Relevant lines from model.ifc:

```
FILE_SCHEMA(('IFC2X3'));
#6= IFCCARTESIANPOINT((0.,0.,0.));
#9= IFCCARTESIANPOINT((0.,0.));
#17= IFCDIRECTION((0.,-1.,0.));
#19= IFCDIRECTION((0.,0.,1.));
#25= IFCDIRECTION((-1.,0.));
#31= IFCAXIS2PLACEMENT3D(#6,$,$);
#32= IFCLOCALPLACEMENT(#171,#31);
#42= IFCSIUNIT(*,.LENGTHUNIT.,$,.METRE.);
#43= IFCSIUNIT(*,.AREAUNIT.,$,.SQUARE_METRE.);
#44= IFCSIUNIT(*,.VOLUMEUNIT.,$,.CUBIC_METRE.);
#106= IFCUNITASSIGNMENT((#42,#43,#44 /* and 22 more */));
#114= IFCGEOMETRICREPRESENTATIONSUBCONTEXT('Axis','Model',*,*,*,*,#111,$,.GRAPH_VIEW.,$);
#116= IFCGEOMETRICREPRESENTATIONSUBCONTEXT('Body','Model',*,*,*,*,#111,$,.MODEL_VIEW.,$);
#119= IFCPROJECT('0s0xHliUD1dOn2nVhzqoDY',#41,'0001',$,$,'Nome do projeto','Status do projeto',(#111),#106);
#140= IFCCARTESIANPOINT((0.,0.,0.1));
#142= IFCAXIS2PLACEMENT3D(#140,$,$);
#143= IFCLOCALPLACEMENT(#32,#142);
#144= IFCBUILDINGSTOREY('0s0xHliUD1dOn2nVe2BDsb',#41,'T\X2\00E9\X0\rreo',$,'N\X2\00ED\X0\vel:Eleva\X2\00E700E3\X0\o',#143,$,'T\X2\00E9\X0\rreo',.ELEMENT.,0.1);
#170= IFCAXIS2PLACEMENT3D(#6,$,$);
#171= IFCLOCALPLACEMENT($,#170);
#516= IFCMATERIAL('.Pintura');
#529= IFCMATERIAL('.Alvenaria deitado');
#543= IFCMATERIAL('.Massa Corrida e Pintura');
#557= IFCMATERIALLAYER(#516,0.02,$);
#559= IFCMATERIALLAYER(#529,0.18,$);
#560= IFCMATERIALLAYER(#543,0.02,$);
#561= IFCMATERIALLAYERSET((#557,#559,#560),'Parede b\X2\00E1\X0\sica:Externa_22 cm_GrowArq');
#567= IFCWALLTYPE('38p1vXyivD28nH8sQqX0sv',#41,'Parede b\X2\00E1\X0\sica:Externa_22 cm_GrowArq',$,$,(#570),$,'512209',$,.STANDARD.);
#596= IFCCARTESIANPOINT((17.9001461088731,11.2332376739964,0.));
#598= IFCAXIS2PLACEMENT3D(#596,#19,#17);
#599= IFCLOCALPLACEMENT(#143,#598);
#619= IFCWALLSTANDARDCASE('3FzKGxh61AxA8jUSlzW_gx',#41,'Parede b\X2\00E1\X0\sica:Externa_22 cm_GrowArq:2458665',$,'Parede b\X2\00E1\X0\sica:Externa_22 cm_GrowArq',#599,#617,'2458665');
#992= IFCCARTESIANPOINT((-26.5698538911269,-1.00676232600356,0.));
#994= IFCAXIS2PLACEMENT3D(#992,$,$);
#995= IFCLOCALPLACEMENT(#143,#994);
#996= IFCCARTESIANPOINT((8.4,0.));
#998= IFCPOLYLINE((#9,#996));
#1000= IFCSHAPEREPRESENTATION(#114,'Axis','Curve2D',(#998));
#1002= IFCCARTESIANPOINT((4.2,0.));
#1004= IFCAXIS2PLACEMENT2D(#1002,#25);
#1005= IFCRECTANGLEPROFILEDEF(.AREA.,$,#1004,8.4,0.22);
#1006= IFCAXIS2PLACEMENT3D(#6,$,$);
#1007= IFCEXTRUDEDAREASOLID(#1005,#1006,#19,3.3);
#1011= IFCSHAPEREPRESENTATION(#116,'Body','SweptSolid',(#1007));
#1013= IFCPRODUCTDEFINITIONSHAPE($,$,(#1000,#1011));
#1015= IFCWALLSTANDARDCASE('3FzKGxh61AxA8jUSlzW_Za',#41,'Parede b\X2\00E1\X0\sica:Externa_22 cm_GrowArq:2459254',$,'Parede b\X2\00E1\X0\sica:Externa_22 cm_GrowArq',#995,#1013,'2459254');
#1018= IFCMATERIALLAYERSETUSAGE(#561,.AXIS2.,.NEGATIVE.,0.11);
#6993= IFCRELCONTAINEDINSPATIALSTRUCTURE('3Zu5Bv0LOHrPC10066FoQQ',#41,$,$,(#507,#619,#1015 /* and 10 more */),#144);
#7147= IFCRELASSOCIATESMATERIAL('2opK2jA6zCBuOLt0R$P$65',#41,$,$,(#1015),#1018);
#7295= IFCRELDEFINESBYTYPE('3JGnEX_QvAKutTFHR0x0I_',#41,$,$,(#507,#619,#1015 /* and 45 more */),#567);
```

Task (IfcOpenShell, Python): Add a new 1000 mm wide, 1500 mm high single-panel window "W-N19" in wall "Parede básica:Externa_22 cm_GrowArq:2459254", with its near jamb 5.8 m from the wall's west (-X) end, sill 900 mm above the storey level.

```python
import numpy as np
import ifcopenshell
import ifcopenshell.api.feature
import ifcopenshell.api.geometry
import ifcopenshell.api.root
import ifcopenshell.api.spatial
import ifcopenshell.api.type
import ifcopenshell.geom
import ifcopenshell.util.element
import ifcopenshell.util.placement
import ifcopenshell.util.representation
import ifcopenshell.util.shape
import ifcopenshell.util.unit

model = ifcopenshell.open("model.ifc")
unit_scale = ifcopenshell.util.unit.calculate_unit_scale(model)
settings = ifcopenshell.geom.settings()


def volume(element):
    """Net volume in cubic metres, openings subtracted."""
    shape = ifcopenshell.geom.create_shape(settings, element)
    return ifcopenshell.util.shape.get_volume(shape.geometry)


wall = model.by_guid("3FzKGxh61AxA8jUSlzW_Za")
storey = ifcopenshell.util.element.get_container(wall, ifc_class="IfcBuildingStorey")
context = ifcopenshell.util.representation.get_context(model, "Model", "Body", "MODEL_VIEW")
before = volume(wall)

width, height, from_end, sill = 1, 1.5, 5.8, 0.9  # metres

# The wall runs along its own X axis, and the end named is its -X end.
wall_shape = ifcopenshell.geom.create_shape(settings, wall)
x, y, z = ifcopenshell.util.shape.get_vertices(wall_shape.geometry).T
start = x.min() + from_end
face, thickness = float(y.min()), float(y.max() - y.min())
wall_matrix = ifcopenshell.util.placement.get_local_placement(wall.ObjectPlacement)
level = ifcopenshell.util.placement.get_local_placement(storey.ObjectPlacement)[2, 3]


def in_wall(x, y):
    """Placement at x, y metres in the wall's axes, at sill height."""
    matrix = wall_matrix.copy()
    matrix[:, 3] = wall_matrix @ np.array([x / unit_scale, y / unit_scale, 0.0, 1.0])
    matrix[2, 3] = level + sill / unit_scale
    return matrix


# Opening: a box that overshoots both wall faces by 50 mm.
opening = ifcopenshell.api.root.create_entity(model, ifc_class="IfcOpeningElement")
box = ifcopenshell.api.geometry.add_wall_representation(
    model, context=context, length=width, height=height, thickness=thickness + 0.1
)
ifcopenshell.api.geometry.assign_representation(model, product=opening, representation=box)
ifcopenshell.api.geometry.edit_object_placement(model, product=opening, matrix=in_wall(start, face - 0.05), is_si=False)
ifcopenshell.api.feature.add_feature(model, feature=opening, element=wall)

window = ifcopenshell.api.root.create_entity(model, ifc_class="IfcWindow", name="W-N19")
window.OverallWidth, window.OverallHeight = width / unit_scale, height / unit_scale
body = ifcopenshell.api.geometry.add_window_representation(
    model,
    context=context,
    overall_width=window.OverallWidth,
    overall_height=window.OverallHeight,
    partition_type="SINGLE_PANEL",
)
ifcopenshell.api.geometry.assign_representation(model, product=window, representation=body)
ifcopenshell.api.spatial.assign_container(model, products=[window], relating_structure=storey)
fills = ifcopenshell.api.feature.add_filling(model, opening=opening, element=window)
fills.OwnerHistory = window.OwnerHistory  # required in IFC2X3

# IFC2X3 keeps the operation on the window style.
style = ifcopenshell.api.root.create_entity(model, ifc_class="IfcWindowStyle", name="W-N19")
style.OperationType, style.ConstructionType = "SINGLE_PANEL", "NOTDEFINED"
style.ParameterTakesPrecedence = style.Sizeable = False
ifcopenshell.api.type.assign_type(model, related_objects=[window], relating_type=style)

# Centre the window in the wall's thickness.
ifcopenshell.api.geometry.edit_object_placement(model, product=window, matrix=in_wall(start, face), is_si=False)
window_shape = ifcopenshell.geom.create_shape(settings, window)
depth = ifcopenshell.util.shape.get_vertices(window_shape.geometry)[:, 1]
offset = face + thickness / 2 - (depth.min() + depth.max()) / 2
ifcopenshell.api.geometry.edit_object_placement(model, product=window, matrix=in_wall(start, offset), is_si=False)

after = volume(wall)

print(f"wall volume {before:.3f} -> {after:.3f} m3")

model.write("model_updated.ifc")
```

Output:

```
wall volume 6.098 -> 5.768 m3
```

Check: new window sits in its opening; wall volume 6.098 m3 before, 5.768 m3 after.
